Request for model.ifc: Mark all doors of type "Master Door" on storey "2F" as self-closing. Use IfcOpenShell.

First a look at what the model holds.

```python
import ifcopenshell
import ifcopenshell.util.element

model = ifcopenshell.open("model.ifc")
print(model.schema)
storey = next(s for s in model.by_type("IfcBuildingStorey") if s.Name == "2F")
doors = [e for e in ifcopenshell.util.element.get_decomposition(storey) if e.is_a("IfcDoor")]
seen = {}
for e in doors:
    element_type = ifcopenshell.util.element.get_type(e)
    key = (element_type.Name if element_type != e and element_type else None, ifcopenshell.util.element.get_pset(e, "Pset_DoorCommon", "SelfClosing"))
    seen[key] = seen.get(key, 0) + 1
for (name, value), count in sorted(seen.items(), key=str):
    print(count, "x", name, "|", value)
```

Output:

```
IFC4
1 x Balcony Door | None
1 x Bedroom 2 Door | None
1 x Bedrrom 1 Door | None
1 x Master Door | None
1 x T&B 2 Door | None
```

```python
import ifcopenshell
import ifcopenshell.api.pset
import ifcopenshell.util.element

model = ifcopenshell.open("model.ifc")

storey = next(s for s in model.by_type("IfcBuildingStorey") if s.Name == "2F")
doors = [e for e in ifcopenshell.util.element.get_decomposition(storey) if e.is_a("IfcDoor")]

count = 0
for e in doors:
    element_type = ifcopenshell.util.element.get_type(e)
    if element_type in (None, e) or element_type.Name != "Master Door":
        continue
    # add_pset returns the element's existing set when there is one.
    pset = ifcopenshell.api.pset.add_pset(model, product=e, name="Pset_DoorCommon")
    ifcopenshell.api.pset.edit_pset(model, pset=pset, properties={"SelfClosing": True})
    count += 1

print(count, "doors updated")

model.write("model_edited.ifc")
```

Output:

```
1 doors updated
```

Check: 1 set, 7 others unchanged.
